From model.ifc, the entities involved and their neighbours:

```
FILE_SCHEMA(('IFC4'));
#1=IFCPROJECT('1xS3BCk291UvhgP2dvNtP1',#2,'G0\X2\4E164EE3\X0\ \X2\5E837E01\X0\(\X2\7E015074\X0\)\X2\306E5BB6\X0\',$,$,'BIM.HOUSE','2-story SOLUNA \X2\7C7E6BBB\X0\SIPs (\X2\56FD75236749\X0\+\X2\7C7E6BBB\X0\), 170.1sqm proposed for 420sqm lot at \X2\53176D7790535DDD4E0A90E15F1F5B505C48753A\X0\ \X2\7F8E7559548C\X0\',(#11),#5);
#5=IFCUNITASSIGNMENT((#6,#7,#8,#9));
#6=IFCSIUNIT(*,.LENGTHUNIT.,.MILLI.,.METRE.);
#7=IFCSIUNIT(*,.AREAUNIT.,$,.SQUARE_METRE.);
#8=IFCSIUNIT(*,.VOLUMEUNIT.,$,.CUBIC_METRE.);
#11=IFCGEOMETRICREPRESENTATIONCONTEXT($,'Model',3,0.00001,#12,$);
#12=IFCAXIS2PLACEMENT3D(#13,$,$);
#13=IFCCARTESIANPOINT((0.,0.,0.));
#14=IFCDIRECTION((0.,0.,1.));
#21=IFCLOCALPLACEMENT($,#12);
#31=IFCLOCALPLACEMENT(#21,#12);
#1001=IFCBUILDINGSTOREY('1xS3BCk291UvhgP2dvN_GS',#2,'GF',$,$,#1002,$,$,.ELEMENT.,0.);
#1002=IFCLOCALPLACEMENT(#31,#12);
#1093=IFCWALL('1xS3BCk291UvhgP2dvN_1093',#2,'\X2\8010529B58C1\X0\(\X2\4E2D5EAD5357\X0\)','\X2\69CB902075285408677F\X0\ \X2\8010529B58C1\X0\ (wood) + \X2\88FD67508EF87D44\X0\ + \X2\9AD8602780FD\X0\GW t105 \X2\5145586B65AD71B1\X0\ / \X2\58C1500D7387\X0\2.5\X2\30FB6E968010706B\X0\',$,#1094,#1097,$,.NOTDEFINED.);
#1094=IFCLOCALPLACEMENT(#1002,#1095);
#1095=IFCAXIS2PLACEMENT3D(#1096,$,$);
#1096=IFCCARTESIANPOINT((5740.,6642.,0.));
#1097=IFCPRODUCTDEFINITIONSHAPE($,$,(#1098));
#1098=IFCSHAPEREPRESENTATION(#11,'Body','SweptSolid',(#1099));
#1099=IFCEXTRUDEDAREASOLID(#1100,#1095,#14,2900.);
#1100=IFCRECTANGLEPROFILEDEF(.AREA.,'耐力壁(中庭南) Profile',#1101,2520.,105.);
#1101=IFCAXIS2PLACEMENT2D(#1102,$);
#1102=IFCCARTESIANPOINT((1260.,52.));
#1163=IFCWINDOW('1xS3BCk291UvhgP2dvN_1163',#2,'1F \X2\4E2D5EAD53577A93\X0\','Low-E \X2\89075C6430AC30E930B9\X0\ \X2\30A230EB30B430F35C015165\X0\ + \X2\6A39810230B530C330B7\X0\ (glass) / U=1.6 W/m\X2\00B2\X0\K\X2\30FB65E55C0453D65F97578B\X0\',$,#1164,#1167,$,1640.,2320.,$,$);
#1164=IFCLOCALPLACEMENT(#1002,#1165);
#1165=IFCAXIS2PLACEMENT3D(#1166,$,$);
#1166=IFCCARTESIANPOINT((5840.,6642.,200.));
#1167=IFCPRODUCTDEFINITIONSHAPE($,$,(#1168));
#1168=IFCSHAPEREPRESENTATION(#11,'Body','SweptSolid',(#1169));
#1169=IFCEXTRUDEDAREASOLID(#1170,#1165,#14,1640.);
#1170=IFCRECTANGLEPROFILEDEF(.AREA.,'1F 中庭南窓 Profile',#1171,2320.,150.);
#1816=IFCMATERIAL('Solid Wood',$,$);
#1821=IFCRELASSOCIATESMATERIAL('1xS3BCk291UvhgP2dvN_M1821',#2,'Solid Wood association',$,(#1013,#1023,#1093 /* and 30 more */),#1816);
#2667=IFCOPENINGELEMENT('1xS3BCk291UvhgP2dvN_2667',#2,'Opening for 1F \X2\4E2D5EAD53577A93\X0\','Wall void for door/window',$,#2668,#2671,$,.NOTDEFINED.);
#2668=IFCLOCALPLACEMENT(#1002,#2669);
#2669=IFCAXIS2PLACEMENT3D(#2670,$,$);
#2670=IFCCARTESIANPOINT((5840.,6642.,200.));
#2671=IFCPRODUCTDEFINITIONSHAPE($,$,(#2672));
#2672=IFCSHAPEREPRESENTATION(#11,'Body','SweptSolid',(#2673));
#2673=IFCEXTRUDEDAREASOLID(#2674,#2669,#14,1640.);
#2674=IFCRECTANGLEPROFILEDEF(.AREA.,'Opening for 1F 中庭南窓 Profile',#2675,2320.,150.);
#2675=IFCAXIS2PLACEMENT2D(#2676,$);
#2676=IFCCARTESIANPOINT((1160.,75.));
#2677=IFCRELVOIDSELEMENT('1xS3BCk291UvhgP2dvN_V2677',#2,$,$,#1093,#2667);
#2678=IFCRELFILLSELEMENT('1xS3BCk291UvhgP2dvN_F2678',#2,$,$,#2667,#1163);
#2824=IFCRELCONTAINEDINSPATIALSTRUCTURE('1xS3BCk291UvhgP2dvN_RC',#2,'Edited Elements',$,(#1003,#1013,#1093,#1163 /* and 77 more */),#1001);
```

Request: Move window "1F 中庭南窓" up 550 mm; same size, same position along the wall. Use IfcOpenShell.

```python
import numpy as np
import ifcopenshell
import ifcopenshell.api.geometry
import ifcopenshell.util.placement
import ifcopenshell.util.unit

model = ifcopenshell.open("model.ifc")
unit_scale = ifcopenshell.util.unit.calculate_unit_scale(model)

window = model.by_id(1163)
opening = window.FillsVoids[0].RelatingOpeningElement
dz = 0.55 / unit_scale

shift = np.array([0.0, 0.0, dz])
# The window is not placed relative to its opening, so move both.
for product in (opening, window):
    matrix = ifcopenshell.util.placement.get_local_placement(product.ObjectPlacement)
    matrix[:3, 3] += shift
    ifcopenshell.api.geometry.edit_object_placement(model, product=product, matrix=matrix, is_si=False)

print(f"moved by {dz * unit_scale:+.3f} m")

model.write("model_v2.ifc")
```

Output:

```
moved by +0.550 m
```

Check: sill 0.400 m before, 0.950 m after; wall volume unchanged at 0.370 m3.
